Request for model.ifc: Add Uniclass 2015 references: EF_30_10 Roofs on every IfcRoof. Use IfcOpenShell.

First a look at what the model holds.

```python
import ifcopenshell

model = ifcopenshell.open("model.ifc")
print(model.schema)
print("classifications:", [c.Name for c in model.by_type("IfcClassification")])
for ifc_class in ("IfcDoor", "IfcRoof", "IfcStair", "IfcWall", "IfcWindow"):
    print(ifc_class, len(model.by_type(ifc_class)))
```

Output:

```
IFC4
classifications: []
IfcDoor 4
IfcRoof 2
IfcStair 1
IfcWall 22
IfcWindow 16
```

```python
import ifcopenshell
import ifcopenshell.api.classification

model = ifcopenshell.open("model.ifc")

system = ifcopenshell.api.classification.add_classification(model, classification="Uniclass 2015")

codes = {
    "IfcRoof": ("EF_30_10", "Roofs"),
}
for ifc_class, (code, name) in codes.items():
    products = model.by_type(ifc_class)
    ifcopenshell.api.classification.add_reference(
        model, products=products, classification=system, identification=code, name=name
    )
    print(code, len(products))

model.write("model_edited.ifc")
```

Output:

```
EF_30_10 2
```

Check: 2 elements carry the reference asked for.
